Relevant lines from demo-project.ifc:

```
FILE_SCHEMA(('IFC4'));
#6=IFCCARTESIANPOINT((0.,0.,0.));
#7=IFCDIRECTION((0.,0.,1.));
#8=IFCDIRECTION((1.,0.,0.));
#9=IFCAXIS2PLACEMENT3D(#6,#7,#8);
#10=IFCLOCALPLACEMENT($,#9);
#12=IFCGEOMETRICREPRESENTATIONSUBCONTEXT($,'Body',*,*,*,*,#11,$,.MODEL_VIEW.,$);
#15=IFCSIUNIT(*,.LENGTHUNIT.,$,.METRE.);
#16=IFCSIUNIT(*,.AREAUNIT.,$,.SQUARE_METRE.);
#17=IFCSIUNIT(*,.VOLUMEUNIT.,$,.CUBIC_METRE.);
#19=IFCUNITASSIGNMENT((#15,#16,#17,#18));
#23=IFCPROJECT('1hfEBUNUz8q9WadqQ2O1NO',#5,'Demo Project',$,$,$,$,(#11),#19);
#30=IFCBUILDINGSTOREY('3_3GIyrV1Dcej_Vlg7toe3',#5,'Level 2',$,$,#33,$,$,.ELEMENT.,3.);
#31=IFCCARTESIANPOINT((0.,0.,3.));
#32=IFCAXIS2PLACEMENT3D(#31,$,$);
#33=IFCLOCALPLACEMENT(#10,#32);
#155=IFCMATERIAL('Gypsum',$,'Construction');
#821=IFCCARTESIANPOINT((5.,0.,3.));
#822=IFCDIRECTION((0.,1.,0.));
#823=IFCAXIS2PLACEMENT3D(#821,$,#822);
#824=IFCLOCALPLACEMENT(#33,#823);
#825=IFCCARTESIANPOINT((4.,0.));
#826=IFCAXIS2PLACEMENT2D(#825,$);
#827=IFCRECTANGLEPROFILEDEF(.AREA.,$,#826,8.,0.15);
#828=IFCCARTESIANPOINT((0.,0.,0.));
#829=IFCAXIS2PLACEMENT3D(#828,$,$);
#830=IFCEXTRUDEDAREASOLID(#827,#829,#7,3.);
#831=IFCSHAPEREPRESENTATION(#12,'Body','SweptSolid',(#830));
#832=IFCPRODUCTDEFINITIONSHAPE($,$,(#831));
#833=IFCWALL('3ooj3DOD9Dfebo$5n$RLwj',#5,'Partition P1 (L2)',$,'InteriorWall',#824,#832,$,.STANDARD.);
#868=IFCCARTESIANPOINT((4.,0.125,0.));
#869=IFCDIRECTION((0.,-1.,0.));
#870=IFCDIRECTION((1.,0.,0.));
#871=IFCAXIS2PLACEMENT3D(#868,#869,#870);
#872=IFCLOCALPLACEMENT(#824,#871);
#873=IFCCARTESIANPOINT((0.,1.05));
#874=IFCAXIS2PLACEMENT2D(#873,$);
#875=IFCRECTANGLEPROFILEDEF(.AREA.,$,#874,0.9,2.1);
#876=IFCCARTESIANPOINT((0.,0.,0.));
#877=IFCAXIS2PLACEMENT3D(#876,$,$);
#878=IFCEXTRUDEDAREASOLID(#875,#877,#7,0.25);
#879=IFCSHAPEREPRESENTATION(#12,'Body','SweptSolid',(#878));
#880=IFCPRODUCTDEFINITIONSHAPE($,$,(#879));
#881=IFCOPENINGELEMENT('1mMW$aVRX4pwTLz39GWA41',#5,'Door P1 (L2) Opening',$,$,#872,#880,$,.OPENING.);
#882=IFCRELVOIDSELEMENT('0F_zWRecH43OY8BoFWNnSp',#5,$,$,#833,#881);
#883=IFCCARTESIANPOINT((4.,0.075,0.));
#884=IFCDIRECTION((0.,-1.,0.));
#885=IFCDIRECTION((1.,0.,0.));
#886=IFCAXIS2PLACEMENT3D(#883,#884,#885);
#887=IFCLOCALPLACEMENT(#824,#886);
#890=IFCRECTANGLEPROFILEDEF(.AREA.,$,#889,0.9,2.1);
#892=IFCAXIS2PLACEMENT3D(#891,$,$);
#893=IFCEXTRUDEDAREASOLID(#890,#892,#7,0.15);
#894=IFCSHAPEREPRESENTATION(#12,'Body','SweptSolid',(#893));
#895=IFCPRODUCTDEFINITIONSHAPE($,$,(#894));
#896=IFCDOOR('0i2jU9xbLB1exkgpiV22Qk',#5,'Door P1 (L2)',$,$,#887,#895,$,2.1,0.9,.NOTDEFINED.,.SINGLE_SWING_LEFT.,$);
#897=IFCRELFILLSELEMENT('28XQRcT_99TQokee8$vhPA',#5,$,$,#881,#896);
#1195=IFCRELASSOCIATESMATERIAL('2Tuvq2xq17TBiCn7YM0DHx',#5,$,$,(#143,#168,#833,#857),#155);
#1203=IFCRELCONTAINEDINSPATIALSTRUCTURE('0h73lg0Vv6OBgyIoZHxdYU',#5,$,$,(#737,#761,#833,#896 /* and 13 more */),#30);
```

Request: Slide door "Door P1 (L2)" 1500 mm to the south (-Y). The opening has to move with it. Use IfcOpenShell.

```python
import ifcopenshell
import ifcopenshell.api.geometry
import ifcopenshell.util.placement

model = ifcopenshell.open("demo-project.ifc")

door = model.by_guid("0i2jU9xbLB1exkgpiV22Qk")
opening = door.FillsVoids[0].RelatingOpeningElement
wall = opening.VoidsElements[0].RelatingBuildingElement

wall_matrix = ifcopenshell.util.placement.get_local_placement(wall.ObjectPlacement)
shift = wall_matrix[:3, 0] * -1.5
before = ifcopenshell.util.placement.get_local_placement(door.ObjectPlacement)[:3, 3].copy()

# The door is not placed relative to its opening, so move both.
for product in (opening, door):
    matrix = ifcopenshell.util.placement.get_local_placement(product.ObjectPlacement)
    matrix[:3, 3] += shift
    ifcopenshell.api.geometry.edit_object_placement(model, product=product, matrix=matrix, is_si=False)

after = ifcopenshell.util.placement.get_local_placement(door.ObjectPlacement)[:3, 3]
print("door moved by", (after - before).round(3) + 0.0)

model.write("demo-project_rev.ifc")
```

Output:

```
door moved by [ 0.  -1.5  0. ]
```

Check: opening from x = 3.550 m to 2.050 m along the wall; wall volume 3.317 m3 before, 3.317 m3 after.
